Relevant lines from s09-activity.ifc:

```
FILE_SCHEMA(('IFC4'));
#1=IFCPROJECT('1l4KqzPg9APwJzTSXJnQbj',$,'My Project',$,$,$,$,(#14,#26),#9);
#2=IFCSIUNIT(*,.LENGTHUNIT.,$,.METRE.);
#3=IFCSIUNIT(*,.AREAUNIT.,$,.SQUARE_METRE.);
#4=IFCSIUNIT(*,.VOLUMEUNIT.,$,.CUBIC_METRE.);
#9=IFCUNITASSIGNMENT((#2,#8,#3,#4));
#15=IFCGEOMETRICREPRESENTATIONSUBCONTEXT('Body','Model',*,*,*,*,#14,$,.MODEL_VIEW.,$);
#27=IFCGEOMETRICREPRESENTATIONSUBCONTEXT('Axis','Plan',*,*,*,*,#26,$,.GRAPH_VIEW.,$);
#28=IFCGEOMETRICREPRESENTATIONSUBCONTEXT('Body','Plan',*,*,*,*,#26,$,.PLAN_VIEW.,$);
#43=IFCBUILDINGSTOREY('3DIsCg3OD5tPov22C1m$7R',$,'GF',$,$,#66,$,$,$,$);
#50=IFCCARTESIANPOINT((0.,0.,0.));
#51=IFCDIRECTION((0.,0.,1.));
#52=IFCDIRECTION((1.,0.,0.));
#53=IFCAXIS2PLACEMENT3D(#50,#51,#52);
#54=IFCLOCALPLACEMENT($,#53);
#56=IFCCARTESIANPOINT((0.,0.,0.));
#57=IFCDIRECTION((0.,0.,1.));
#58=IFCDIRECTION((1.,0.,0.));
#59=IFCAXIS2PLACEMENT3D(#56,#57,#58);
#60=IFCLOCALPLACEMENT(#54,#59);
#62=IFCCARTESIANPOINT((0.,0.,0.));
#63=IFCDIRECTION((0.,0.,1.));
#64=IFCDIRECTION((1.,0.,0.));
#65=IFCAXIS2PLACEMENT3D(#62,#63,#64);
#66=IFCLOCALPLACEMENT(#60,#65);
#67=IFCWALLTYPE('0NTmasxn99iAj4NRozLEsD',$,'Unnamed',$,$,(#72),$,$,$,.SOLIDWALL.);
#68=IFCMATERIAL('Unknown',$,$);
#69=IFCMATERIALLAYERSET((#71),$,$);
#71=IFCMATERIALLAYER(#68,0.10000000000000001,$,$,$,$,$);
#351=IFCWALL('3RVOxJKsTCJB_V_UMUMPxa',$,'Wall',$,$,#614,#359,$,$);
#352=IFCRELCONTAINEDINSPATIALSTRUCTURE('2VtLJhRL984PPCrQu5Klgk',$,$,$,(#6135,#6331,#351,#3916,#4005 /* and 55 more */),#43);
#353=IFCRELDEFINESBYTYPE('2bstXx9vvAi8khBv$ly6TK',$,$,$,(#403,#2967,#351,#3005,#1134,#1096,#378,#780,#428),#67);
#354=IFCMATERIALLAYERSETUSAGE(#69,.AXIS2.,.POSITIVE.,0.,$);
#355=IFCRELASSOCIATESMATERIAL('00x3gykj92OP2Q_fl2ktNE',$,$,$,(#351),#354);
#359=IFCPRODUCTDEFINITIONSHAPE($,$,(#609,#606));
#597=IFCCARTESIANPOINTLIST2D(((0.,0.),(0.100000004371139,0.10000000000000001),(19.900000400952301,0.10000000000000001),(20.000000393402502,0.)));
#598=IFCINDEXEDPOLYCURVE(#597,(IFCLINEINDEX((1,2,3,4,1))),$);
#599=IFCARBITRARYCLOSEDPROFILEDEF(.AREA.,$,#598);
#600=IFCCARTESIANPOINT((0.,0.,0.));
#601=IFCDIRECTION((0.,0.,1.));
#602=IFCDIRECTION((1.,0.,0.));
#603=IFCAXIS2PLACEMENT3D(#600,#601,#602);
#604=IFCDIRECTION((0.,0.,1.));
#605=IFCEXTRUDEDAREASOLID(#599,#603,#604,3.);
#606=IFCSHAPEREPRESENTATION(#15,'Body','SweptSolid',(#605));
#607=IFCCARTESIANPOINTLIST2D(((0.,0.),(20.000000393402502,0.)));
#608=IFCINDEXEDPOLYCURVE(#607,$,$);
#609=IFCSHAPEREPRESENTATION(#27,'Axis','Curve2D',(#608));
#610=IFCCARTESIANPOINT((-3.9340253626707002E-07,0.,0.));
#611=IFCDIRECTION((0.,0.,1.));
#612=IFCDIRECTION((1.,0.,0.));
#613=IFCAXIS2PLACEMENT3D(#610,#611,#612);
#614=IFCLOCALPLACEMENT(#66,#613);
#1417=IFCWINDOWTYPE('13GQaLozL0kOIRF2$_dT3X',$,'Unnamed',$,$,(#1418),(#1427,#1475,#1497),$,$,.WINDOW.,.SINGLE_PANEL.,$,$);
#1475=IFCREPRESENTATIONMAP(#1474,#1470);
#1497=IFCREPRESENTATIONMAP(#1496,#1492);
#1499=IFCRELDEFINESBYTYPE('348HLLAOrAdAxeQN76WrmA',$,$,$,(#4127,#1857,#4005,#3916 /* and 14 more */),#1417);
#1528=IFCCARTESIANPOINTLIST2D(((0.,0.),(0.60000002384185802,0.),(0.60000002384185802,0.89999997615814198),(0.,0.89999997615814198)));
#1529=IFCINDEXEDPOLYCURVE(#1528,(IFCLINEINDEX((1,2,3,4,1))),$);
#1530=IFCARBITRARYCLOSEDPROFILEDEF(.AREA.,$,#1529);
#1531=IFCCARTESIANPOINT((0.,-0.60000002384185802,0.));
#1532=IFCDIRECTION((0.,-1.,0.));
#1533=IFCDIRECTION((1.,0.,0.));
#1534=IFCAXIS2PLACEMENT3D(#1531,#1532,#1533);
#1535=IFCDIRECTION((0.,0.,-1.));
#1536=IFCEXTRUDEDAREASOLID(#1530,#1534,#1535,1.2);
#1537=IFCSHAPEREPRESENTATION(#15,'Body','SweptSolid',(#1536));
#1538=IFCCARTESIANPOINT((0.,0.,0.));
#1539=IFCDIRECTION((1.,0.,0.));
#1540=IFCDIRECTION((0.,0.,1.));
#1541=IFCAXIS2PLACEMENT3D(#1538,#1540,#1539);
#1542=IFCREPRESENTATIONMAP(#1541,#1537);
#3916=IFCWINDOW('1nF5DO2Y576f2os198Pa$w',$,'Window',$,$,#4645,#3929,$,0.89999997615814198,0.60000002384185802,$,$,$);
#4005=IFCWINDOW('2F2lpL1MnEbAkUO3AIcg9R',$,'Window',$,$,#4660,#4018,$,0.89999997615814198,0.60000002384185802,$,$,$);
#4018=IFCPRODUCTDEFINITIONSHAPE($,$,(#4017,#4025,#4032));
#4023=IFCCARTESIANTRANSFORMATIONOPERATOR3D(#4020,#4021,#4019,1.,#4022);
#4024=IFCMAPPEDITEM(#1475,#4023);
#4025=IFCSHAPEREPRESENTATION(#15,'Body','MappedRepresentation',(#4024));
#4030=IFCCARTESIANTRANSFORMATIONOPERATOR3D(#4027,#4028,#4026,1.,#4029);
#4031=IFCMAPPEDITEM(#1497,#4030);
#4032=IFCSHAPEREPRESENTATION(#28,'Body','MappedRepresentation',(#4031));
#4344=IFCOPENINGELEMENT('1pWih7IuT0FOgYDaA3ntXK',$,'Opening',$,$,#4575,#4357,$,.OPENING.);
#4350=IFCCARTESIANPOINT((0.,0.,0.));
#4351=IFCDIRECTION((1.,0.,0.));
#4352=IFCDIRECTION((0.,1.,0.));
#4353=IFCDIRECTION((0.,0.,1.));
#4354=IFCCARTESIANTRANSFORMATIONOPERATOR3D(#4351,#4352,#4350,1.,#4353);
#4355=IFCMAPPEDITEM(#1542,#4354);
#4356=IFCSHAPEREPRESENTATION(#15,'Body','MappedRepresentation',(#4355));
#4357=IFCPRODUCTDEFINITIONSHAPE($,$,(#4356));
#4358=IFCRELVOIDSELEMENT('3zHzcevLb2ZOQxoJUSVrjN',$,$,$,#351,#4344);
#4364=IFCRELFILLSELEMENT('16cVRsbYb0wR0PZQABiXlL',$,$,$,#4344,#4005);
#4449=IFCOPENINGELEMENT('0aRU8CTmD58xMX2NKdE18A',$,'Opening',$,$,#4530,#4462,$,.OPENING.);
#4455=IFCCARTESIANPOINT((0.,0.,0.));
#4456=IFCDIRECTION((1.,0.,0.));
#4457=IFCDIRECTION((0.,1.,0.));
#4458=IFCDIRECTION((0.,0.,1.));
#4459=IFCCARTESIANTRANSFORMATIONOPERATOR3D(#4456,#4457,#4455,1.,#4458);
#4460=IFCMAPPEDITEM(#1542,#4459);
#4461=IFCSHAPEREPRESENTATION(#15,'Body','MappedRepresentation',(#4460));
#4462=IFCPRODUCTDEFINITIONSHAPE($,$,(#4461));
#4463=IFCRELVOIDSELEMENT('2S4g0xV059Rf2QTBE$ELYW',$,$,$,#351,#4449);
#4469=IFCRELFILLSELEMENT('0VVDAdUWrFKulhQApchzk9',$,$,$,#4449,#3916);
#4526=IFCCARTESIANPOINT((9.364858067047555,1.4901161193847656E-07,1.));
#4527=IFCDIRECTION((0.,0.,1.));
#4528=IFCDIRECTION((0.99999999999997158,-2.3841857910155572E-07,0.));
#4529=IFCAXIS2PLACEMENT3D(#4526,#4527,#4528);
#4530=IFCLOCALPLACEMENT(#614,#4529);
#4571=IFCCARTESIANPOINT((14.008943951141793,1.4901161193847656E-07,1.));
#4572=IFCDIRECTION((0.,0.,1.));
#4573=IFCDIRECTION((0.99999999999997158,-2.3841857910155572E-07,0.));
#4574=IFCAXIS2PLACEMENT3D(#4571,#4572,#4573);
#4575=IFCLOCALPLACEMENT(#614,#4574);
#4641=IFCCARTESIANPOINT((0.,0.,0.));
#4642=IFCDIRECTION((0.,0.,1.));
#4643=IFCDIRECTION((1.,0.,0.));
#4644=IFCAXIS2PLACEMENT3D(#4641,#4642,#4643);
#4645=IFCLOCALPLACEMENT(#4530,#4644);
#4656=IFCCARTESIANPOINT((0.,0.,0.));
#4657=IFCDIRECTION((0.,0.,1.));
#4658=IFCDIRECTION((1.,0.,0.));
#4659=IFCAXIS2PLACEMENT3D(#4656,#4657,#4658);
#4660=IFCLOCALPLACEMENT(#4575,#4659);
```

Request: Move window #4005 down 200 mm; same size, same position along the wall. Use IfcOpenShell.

```python
import numpy as np
import ifcopenshell
import ifcopenshell.api.geometry
import ifcopenshell.util.placement
import ifcopenshell.util.unit

model = ifcopenshell.open("s09-activity.ifc")
unit_scale = ifcopenshell.util.unit.calculate_unit_scale(model)

window = model.by_id(4005)
opening = window.FillsVoids[0].RelatingOpeningElement
dz = -0.2 / unit_scale

shift = np.array([0.0, 0.0, dz])
# The window is placed relative to its opening, so it follows when the opening moves.
matrix = ifcopenshell.util.placement.get_local_placement(opening.ObjectPlacement)
matrix[:3, 3] += shift
ifcopenshell.api.geometry.edit_object_placement(
    model, product=opening, matrix=matrix, is_si=False, should_transform_children=True
)

print(f"moved by {dz * unit_scale:+.3f} m")

model.write("s09-activity_updated.ifc")
```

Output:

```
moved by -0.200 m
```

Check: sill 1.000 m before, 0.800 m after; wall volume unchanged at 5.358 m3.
